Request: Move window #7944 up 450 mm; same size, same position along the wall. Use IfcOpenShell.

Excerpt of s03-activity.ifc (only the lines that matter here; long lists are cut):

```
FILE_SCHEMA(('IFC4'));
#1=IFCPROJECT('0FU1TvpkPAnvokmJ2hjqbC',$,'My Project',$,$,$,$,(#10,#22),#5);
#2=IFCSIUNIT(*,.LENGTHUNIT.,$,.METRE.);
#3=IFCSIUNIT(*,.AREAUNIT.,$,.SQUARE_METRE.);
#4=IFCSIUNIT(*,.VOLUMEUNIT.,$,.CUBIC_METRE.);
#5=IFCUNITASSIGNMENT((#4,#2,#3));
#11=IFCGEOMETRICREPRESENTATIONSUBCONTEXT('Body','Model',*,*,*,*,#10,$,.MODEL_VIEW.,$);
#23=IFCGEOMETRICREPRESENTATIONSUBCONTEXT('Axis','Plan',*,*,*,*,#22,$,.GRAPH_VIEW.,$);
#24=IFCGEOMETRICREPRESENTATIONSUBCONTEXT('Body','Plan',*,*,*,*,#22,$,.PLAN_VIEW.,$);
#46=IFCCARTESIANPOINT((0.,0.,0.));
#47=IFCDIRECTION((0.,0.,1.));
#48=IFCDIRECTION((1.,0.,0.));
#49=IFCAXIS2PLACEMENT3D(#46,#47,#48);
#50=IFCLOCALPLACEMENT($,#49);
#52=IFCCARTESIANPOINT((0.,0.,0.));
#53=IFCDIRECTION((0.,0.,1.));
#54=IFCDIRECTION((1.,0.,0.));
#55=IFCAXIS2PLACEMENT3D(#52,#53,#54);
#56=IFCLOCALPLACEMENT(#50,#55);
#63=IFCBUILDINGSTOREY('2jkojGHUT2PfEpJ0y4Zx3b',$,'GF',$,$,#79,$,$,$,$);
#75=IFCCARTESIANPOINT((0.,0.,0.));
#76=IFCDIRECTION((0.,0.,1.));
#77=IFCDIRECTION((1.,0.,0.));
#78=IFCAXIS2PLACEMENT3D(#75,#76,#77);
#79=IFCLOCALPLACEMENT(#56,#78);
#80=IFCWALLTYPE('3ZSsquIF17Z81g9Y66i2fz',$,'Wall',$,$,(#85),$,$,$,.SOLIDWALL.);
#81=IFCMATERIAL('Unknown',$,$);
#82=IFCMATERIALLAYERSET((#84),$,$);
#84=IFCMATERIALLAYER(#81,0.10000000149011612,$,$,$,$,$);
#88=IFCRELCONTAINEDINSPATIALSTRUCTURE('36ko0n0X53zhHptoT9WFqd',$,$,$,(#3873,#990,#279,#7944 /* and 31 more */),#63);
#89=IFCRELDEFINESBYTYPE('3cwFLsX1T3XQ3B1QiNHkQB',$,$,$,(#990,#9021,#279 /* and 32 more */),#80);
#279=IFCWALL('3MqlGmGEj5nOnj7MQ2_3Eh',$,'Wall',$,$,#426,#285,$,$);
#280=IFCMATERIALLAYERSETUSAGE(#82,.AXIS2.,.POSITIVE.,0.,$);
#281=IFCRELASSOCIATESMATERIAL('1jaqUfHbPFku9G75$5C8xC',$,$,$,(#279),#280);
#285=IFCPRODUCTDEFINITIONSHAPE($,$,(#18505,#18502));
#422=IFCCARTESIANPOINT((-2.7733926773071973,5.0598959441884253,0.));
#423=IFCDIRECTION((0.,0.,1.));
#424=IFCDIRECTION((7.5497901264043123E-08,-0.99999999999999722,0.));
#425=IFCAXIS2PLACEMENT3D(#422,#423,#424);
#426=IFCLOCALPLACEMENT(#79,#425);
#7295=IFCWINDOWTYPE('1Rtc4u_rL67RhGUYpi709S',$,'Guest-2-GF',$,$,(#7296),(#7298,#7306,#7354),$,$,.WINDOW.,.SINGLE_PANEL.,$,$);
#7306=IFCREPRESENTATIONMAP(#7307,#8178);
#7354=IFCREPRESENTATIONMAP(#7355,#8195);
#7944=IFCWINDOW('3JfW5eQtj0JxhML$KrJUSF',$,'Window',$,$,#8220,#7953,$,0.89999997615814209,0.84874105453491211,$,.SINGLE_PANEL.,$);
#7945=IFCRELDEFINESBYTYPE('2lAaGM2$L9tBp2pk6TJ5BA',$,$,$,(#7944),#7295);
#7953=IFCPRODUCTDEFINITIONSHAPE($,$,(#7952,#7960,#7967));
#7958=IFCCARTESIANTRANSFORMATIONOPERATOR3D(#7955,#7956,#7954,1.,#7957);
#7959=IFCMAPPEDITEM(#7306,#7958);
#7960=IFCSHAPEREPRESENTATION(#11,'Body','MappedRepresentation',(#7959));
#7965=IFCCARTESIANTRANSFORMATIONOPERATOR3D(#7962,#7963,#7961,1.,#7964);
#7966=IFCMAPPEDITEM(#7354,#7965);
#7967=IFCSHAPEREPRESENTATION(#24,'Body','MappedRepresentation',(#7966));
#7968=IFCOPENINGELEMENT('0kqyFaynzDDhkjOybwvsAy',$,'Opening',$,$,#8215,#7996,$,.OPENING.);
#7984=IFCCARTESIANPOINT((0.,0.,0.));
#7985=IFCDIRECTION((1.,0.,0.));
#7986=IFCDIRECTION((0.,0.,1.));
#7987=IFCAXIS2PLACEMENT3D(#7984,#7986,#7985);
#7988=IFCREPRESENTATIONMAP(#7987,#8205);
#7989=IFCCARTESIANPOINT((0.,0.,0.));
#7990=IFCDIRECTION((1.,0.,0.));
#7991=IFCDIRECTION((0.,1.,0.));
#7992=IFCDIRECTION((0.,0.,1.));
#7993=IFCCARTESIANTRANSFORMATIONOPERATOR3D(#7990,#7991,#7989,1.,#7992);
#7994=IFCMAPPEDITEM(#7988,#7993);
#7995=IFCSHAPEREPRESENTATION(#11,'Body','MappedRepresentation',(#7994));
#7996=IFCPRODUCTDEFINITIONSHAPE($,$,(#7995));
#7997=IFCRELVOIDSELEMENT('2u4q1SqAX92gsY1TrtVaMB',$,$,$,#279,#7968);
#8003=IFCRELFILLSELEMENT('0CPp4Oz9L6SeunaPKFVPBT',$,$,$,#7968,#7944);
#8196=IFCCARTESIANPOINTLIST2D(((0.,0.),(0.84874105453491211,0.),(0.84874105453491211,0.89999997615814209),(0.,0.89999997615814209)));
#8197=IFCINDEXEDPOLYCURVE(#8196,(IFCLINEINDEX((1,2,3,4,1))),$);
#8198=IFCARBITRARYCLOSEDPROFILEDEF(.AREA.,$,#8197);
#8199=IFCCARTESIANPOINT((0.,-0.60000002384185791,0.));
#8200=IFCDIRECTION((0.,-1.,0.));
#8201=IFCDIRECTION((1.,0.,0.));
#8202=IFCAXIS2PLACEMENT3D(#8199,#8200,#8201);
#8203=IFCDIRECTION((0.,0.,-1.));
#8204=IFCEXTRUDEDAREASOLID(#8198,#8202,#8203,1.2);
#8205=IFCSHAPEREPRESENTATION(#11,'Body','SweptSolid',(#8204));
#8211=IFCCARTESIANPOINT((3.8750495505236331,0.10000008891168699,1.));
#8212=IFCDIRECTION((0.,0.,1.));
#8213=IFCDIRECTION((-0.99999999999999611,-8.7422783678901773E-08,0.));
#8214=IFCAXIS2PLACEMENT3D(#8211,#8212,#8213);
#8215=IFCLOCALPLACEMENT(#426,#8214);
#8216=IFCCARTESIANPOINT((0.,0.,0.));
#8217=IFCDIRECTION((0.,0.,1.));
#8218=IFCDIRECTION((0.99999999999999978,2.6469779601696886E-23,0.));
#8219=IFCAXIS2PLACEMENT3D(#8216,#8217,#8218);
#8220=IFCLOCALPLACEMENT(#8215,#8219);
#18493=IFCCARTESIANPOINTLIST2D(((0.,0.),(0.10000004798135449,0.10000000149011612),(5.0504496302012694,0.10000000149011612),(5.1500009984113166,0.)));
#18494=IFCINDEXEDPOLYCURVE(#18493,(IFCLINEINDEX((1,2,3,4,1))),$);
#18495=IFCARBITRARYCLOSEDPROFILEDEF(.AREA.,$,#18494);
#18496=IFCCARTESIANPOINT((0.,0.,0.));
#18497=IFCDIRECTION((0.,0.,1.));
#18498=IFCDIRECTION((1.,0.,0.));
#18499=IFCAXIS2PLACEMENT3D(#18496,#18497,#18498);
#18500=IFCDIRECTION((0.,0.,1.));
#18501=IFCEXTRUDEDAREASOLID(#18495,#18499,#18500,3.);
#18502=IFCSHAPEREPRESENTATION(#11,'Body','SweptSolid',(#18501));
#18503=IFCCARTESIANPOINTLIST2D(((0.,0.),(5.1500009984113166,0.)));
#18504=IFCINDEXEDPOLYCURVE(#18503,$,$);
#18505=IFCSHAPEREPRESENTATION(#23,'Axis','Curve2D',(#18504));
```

```python
import numpy as np
import ifcopenshell
import ifcopenshell.api.geometry
import ifcopenshell.util.placement
import ifcopenshell.util.unit

model = ifcopenshell.open("s03-activity.ifc")
unit_scale = ifcopenshell.util.unit.calculate_unit_scale(model)

window = model.by_id(7944)
opening = window.FillsVoids[0].RelatingOpeningElement
dz = 0.45

shift = np.array([0.0, 0.0, dz])
# The window is placed relative to its opening, so it follows when the opening moves.
matrix = ifcopenshell.util.placement.get_local_placement(opening.ObjectPlacement)
matrix[:3, 3] += shift
ifcopenshell.api.geometry.edit_object_placement(
    model, product=opening, matrix=matrix, is_si=False, should_transform_children=True
)

print(f"moved by {dz * unit_scale:+.3f} m")

model.write("s03-activity-out.ifc")
```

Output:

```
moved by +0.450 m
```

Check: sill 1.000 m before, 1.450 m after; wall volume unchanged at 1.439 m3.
